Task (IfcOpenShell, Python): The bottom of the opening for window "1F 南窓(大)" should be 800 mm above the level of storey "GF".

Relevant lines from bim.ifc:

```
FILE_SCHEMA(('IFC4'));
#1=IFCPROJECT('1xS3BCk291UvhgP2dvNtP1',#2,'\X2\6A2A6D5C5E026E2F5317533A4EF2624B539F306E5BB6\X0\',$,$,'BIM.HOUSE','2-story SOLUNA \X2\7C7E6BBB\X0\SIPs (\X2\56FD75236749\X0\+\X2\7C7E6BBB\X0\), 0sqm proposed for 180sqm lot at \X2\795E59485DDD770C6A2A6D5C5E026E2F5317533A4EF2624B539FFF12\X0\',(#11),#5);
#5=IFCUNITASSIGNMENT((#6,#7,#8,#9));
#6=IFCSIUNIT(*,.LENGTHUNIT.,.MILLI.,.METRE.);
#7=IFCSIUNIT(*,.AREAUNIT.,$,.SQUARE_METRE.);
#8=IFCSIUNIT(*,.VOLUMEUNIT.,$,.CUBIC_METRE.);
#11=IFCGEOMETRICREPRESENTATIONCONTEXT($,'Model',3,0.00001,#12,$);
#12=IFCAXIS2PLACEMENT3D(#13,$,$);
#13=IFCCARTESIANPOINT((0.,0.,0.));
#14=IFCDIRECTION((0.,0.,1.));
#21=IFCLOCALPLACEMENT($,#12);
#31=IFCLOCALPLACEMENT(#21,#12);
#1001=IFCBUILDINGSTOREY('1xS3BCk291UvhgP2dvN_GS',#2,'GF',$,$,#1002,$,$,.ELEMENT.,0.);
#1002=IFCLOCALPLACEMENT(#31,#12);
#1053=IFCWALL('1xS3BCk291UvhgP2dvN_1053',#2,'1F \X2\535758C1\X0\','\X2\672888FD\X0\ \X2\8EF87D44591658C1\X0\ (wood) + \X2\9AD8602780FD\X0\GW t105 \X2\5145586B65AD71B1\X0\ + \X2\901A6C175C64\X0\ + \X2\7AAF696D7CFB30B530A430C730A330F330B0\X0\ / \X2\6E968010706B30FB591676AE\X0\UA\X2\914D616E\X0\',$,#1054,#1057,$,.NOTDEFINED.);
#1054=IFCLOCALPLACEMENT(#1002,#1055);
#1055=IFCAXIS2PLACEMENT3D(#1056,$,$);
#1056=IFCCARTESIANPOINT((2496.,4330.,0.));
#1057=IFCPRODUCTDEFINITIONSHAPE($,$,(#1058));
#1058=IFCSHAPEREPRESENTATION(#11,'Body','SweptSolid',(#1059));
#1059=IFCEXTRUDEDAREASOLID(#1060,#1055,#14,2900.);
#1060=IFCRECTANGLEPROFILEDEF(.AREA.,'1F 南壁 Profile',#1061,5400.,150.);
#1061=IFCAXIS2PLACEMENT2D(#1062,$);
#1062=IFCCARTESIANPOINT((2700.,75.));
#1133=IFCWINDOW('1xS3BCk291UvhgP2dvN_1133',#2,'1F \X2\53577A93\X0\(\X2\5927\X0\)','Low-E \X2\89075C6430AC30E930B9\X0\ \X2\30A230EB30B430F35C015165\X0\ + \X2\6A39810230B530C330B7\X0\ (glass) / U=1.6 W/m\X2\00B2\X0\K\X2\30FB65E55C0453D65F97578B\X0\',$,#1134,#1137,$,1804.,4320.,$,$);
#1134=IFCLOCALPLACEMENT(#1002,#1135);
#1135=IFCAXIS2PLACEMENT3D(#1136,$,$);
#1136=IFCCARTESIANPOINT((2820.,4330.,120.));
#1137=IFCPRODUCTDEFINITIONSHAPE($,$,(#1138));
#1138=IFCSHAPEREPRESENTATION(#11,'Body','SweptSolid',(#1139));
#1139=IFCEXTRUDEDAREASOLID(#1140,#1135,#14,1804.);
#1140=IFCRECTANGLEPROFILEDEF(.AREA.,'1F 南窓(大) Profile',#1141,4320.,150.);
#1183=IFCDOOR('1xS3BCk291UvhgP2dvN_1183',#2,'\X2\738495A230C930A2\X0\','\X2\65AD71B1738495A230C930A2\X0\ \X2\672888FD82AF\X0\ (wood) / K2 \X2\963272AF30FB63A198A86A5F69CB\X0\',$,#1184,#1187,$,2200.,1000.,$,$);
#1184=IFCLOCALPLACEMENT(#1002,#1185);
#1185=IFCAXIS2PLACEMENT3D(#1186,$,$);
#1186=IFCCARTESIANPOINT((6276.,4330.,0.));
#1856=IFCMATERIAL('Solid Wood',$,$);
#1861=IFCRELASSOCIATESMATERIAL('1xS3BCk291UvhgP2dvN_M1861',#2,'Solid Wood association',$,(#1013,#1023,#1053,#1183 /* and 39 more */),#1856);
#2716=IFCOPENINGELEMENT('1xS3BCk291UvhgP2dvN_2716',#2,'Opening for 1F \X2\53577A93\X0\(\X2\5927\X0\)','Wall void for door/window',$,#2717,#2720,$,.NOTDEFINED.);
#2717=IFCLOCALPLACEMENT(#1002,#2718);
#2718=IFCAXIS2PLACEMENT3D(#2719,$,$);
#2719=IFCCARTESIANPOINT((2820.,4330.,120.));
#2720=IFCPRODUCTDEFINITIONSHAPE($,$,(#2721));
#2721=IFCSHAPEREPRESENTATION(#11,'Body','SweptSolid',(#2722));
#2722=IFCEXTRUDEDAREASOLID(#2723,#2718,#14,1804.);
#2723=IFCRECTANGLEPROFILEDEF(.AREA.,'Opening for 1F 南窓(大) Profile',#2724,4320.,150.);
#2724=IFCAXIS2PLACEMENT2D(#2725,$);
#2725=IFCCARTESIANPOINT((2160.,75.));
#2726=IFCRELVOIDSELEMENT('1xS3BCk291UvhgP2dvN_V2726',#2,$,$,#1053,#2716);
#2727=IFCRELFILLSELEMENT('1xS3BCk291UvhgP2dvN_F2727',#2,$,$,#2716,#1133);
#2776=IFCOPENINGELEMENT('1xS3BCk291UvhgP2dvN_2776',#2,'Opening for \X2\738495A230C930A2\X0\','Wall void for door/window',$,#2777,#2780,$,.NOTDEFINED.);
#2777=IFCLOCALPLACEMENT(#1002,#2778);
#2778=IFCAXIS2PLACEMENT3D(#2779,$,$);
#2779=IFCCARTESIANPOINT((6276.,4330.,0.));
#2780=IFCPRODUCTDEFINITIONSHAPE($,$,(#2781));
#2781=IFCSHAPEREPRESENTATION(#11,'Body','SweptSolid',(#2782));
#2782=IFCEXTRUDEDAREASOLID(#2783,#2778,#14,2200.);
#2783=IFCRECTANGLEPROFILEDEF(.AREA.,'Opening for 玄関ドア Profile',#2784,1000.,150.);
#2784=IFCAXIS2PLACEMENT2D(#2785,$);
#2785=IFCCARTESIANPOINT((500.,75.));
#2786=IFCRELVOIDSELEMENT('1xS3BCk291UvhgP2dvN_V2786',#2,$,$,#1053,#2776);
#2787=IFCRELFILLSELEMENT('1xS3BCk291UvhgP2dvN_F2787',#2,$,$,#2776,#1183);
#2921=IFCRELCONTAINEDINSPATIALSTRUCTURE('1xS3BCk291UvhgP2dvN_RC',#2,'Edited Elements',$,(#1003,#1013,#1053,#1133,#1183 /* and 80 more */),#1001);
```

```python
import numpy as np
import ifcopenshell
import ifcopenshell.api.geometry
import ifcopenshell.geom
import ifcopenshell.util.element
import ifcopenshell.util.placement
import ifcopenshell.util.shape
import ifcopenshell.util.unit

model = ifcopenshell.open("bim.ifc")
unit_scale = ifcopenshell.util.unit.calculate_unit_scale(model)

window = model.by_guid("1xS3BCk291UvhgP2dvN_1133")
opening = window.FillsVoids[0].RelatingOpeningElement
storey = ifcopenshell.util.element.get_container(window, ifc_class="IfcBuildingStorey")
level = ifcopenshell.util.placement.get_local_placement(storey.ObjectPlacement)[2, 3]

# The opening's origin need not be at the sill, so measure its lowest point.
shape = ifcopenshell.geom.create_shape(ifcopenshell.geom.settings(), opening)
bottom = ifcopenshell.util.shape.get_shape_bottom_elevation(shape, shape.geometry) / unit_scale
dz = level + 0.8 / unit_scale - bottom

shift = np.array([0.0, 0.0, dz])
# The window is not placed relative to its opening, so move both.
for product in (opening, window):
    matrix = ifcopenshell.util.placement.get_local_placement(product.ObjectPlacement)
    matrix[:3, 3] += shift
    ifcopenshell.api.geometry.edit_object_placement(model, product=product, matrix=matrix, is_si=False)

print(f"moved by {dz * unit_scale:+.3f} m")

model.write("bim_rev.ifc")
```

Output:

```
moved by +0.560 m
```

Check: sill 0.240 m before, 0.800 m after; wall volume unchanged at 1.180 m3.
